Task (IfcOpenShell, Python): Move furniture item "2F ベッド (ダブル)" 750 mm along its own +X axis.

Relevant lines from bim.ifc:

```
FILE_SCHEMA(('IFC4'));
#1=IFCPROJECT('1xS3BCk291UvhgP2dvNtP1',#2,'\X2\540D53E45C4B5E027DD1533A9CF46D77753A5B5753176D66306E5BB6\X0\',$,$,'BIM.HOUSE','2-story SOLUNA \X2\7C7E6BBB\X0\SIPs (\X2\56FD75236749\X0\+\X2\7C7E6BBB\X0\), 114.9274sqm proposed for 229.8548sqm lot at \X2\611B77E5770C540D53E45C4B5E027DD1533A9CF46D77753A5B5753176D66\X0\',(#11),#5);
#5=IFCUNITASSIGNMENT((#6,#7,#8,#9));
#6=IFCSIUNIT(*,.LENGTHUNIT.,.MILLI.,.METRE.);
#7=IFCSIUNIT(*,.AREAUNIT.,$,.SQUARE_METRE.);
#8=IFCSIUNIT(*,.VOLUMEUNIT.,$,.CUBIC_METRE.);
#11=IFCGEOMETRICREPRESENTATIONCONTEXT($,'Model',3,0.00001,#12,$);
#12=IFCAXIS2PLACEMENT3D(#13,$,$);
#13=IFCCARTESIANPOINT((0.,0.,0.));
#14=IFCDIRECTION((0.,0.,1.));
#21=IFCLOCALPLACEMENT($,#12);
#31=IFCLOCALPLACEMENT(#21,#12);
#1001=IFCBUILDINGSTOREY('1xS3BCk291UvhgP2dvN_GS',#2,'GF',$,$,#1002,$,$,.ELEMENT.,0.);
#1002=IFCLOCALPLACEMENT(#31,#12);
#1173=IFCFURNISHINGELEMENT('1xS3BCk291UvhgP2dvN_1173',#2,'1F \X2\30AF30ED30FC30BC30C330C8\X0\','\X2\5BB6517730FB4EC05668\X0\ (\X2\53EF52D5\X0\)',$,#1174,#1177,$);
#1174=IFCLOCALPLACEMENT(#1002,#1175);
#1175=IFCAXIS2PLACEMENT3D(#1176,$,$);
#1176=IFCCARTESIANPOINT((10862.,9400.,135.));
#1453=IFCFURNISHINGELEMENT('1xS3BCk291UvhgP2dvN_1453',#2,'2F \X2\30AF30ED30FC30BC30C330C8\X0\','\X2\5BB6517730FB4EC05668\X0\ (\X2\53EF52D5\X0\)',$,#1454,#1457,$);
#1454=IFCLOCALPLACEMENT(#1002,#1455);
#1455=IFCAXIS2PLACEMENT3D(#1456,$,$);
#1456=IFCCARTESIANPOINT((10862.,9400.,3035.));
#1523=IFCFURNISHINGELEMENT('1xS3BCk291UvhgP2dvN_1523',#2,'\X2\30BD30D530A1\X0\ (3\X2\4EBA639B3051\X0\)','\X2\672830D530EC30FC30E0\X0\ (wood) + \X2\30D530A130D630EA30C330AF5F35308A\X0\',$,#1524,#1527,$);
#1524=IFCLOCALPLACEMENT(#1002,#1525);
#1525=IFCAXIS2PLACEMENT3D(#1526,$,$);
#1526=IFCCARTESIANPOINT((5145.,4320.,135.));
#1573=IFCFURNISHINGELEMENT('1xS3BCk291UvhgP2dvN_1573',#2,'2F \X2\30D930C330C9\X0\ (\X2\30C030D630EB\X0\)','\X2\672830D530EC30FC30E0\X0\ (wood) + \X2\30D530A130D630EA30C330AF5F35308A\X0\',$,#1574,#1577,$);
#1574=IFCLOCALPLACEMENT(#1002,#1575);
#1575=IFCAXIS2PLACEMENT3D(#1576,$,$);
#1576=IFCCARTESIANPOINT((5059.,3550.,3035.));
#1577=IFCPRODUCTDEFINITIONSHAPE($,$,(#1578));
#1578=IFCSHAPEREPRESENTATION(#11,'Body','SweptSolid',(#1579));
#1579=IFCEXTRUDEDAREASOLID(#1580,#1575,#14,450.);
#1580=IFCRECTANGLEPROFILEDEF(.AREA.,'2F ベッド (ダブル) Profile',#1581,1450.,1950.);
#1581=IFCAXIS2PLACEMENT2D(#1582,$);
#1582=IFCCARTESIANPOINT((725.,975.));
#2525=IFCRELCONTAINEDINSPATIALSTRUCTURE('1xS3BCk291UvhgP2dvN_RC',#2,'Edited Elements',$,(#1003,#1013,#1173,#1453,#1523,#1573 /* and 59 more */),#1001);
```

```python
import ifcopenshell
import ifcopenshell.api.geometry
import ifcopenshell.util.placement

model = ifcopenshell.open("bim.ifc")

item = model.by_guid("1xS3BCk291UvhgP2dvN_1573")
matrix = ifcopenshell.util.placement.get_local_placement(item.ObjectPlacement)
matrix[:3, 3] += matrix[:3, 0] * 750.0
ifcopenshell.api.geometry.edit_object_placement(model, product=item, matrix=matrix, is_si=False)

print(ifcopenshell.util.placement.get_local_placement(item.ObjectPlacement).round(3) + 0.0)

model.write("bim_v2.ifc")
```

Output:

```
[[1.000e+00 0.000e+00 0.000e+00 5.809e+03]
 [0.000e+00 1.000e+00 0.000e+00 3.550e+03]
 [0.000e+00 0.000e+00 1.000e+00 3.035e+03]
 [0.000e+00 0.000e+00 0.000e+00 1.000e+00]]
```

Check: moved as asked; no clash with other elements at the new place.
